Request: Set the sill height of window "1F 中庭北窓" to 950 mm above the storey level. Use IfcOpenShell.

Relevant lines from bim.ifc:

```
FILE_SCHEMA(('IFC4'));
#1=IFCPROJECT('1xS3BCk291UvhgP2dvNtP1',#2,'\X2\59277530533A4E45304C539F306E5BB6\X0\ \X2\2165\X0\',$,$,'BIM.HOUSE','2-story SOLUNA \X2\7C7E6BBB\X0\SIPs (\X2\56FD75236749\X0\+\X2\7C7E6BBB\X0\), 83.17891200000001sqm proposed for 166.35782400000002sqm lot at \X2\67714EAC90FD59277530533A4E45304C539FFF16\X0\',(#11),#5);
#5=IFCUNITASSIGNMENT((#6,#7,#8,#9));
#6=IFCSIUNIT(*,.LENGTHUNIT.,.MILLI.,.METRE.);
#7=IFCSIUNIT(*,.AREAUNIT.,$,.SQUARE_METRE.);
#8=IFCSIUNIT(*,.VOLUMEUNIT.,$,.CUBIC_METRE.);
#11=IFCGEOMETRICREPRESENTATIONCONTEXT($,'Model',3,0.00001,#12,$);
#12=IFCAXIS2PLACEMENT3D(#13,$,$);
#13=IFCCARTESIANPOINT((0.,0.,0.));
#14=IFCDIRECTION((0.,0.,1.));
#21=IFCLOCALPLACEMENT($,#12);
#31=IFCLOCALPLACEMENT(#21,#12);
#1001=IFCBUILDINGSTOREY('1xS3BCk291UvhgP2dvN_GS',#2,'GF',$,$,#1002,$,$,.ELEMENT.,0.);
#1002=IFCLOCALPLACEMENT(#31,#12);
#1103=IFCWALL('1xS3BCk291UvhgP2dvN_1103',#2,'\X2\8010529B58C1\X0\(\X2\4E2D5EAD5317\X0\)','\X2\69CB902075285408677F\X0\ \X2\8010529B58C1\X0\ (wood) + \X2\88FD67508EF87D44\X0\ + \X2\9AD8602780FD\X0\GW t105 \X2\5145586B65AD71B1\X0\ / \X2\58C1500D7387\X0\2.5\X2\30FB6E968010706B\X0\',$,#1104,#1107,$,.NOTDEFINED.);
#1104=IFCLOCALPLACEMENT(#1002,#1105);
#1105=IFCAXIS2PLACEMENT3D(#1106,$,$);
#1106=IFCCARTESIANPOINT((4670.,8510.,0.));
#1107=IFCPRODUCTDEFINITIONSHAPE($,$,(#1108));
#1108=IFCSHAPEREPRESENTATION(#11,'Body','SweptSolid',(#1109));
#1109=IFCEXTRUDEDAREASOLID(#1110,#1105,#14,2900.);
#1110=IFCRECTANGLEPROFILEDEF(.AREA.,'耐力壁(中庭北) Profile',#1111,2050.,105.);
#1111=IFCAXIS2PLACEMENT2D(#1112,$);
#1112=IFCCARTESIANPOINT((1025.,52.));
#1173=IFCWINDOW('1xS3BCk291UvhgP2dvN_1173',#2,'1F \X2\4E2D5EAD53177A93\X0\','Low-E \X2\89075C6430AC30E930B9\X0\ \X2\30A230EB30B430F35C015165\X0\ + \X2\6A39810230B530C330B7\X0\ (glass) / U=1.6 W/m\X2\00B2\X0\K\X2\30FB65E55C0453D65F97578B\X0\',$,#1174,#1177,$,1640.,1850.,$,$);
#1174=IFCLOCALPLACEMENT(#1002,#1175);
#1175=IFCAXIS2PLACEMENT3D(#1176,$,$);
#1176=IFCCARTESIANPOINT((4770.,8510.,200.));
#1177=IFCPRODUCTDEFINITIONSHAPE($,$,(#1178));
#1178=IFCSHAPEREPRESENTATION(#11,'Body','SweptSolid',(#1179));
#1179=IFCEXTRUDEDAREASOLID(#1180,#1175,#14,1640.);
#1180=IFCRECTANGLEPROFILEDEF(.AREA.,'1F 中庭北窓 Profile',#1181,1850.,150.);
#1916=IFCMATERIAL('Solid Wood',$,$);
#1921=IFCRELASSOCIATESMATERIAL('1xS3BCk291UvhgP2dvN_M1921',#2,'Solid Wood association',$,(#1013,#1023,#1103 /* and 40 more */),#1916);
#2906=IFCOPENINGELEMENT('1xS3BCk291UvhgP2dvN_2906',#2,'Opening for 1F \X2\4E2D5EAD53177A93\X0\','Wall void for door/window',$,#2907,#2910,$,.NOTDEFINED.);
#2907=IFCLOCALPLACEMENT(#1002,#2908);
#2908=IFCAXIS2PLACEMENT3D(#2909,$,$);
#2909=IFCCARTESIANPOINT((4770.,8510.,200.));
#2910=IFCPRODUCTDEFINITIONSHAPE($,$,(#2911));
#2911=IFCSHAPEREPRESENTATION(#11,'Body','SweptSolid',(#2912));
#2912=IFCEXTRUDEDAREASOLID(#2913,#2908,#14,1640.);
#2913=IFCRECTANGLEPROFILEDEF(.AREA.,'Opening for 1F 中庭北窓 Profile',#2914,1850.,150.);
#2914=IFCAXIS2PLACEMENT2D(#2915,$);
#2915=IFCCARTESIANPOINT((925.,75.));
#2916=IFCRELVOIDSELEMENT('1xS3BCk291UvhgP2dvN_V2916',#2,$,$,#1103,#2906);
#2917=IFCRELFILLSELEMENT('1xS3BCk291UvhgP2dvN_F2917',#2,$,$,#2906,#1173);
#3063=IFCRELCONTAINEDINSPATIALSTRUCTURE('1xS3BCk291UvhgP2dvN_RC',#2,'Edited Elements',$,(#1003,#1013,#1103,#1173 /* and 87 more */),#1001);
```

```python
import numpy as np
import ifcopenshell
import ifcopenshell.api.geometry
import ifcopenshell.geom
import ifcopenshell.util.element
import ifcopenshell.util.placement
import ifcopenshell.util.shape
import ifcopenshell.util.unit

model = ifcopenshell.open("bim.ifc")
unit_scale = ifcopenshell.util.unit.calculate_unit_scale(model)

window = model.by_guid("1xS3BCk291UvhgP2dvN_1173")
opening = window.FillsVoids[0].RelatingOpeningElement
storey = ifcopenshell.util.element.get_container(window, ifc_class="IfcBuildingStorey")
level = ifcopenshell.util.placement.get_local_placement(storey.ObjectPlacement)[2, 3]

# The opening's origin need not be at the sill, so measure its lowest point.
shape = ifcopenshell.geom.create_shape(ifcopenshell.geom.settings(), opening)
bottom = ifcopenshell.util.shape.get_shape_bottom_elevation(shape, shape.geometry) / unit_scale
dz = level + 0.95 / unit_scale - bottom

shift = np.array([0.0, 0.0, dz])
# The window is not placed relative to its opening, so move both.
for product in (opening, window):
    matrix = ifcopenshell.util.placement.get_local_placement(product.ObjectPlacement)
    matrix[:3, 3] += shift
    ifcopenshell.api.geometry.edit_object_placement(model, product=product, matrix=matrix, is_si=False)

print(f"moved by {dz * unit_scale:+.3f} m")

model.write("bim_rev.ifc")
```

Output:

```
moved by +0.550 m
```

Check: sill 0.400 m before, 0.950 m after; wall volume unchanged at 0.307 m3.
